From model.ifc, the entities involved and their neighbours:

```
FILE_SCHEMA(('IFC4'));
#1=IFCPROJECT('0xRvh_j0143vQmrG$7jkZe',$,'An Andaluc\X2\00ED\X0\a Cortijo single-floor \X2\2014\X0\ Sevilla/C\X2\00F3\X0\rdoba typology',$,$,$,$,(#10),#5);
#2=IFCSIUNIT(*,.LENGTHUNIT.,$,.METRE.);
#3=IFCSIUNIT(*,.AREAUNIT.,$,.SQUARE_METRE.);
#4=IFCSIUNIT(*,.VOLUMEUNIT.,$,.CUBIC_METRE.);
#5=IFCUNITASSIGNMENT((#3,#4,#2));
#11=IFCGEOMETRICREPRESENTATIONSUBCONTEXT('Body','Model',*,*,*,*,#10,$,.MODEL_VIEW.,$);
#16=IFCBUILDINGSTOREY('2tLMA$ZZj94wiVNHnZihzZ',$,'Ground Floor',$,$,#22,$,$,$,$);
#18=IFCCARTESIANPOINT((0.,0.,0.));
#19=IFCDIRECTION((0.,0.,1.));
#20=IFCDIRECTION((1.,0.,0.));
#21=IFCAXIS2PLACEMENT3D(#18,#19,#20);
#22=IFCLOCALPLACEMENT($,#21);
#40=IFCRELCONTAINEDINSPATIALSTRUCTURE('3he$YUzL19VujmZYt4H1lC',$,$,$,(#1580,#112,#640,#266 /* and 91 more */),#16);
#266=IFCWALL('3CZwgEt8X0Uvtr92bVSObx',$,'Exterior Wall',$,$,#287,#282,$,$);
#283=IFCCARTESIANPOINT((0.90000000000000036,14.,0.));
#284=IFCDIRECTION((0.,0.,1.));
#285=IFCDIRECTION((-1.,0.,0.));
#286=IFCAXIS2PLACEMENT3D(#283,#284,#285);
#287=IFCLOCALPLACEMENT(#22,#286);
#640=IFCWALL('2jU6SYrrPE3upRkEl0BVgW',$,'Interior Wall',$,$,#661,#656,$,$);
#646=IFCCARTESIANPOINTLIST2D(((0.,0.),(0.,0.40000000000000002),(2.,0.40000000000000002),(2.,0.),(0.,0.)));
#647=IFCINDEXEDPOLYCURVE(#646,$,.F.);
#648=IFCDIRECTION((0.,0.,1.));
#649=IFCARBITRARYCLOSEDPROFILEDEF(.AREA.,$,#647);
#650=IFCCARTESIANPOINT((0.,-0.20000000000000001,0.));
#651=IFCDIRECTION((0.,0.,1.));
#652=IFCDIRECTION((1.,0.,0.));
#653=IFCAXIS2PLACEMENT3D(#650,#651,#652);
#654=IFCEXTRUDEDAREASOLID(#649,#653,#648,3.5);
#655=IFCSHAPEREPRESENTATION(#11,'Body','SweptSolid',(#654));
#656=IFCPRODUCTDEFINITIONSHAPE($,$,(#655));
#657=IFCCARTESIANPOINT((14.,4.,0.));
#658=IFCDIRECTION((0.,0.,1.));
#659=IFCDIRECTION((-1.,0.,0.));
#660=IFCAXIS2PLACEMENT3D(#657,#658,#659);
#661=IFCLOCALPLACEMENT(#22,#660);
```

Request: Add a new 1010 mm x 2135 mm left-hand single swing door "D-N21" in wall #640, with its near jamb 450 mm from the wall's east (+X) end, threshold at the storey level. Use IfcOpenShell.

```python
import numpy as np
import ifcopenshell
import ifcopenshell.api.feature
import ifcopenshell.api.geometry
import ifcopenshell.api.root
import ifcopenshell.api.spatial
import ifcopenshell.geom
import ifcopenshell.util.element
import ifcopenshell.util.placement
import ifcopenshell.util.representation
import ifcopenshell.util.shape
import ifcopenshell.util.unit

model = ifcopenshell.open("model.ifc")
unit_scale = ifcopenshell.util.unit.calculate_unit_scale(model)
settings = ifcopenshell.geom.settings()


def volume(element):
    """Net volume in cubic metres, openings subtracted."""
    shape = ifcopenshell.geom.create_shape(settings, element)
    return ifcopenshell.util.shape.get_volume(shape.geometry)


wall = model.by_guid("2jU6SYrrPE3upRkEl0BVgW")
storey = ifcopenshell.util.element.get_container(wall, ifc_class="IfcBuildingStorey")
context = ifcopenshell.util.representation.get_context(model, "Model", "Body", "MODEL_VIEW")
before = volume(wall)

width, height, from_end, sill = 1.01, 2.135, 0.45, 0.0  # metres

# The wall runs along its own X axis, and the end named is its -X end.
wall_shape = ifcopenshell.geom.create_shape(settings, wall)
x, y, z = ifcopenshell.util.shape.get_vertices(wall_shape.geometry).T
start = x.min() + from_end
face, thickness = float(y.min()), float(y.max() - y.min())
wall_matrix = ifcopenshell.util.placement.get_local_placement(wall.ObjectPlacement)
level = ifcopenshell.util.placement.get_local_placement(storey.ObjectPlacement)[2, 3]


def in_wall(x, y):
    """Placement at x, y metres in the wall's axes, at sill height."""
    matrix = wall_matrix.copy()
    matrix[:, 3] = wall_matrix @ np.array([x / unit_scale, y / unit_scale, 0.0, 1.0])
    matrix[2, 3] = level + sill / unit_scale
    return matrix


# Opening: a box that overshoots both wall faces by 50 mm.
opening = ifcopenshell.api.root.create_entity(model, ifc_class="IfcOpeningElement", predefined_type="OPENING")
box = ifcopenshell.api.geometry.add_wall_representation(
    model, context=context, length=width, height=height, thickness=thickness + 0.1
)
ifcopenshell.api.geometry.assign_representation(model, product=opening, representation=box)
ifcopenshell.api.geometry.edit_object_placement(model, product=opening, matrix=in_wall(start, face - 0.05), is_si=False)
ifcopenshell.api.feature.add_feature(model, feature=opening, element=wall)

door = ifcopenshell.api.root.create_entity(model, ifc_class="IfcDoor", name="D-N21", predefined_type="DOOR")
door.OverallWidth, door.OverallHeight = width / unit_scale, height / unit_scale
door.OperationType = "SINGLE_SWING_LEFT"
body = ifcopenshell.api.geometry.add_door_representation(
    model,
    context=context,
    overall_width=door.OverallWidth,
    overall_height=door.OverallHeight,
    operation_type="SINGLE_SWING_LEFT",
    lining_properties={"LiningDepth": thickness / unit_scale, "ThresholdDepth": thickness / unit_scale},
)
ifcopenshell.api.geometry.assign_representation(model, product=door, representation=body)
ifcopenshell.api.spatial.assign_container(model, products=[door], relating_structure=storey)
ifcopenshell.api.feature.add_filling(model, opening=opening, element=door)

# The lining spans the wall, so the door starts at the wall face.
ifcopenshell.api.geometry.edit_object_placement(model, product=door, matrix=in_wall(start, face), is_si=False)

after = volume(wall)

print(f"wall volume {before:.3f} -> {after:.3f} m3")

model.write("model-out.ifc")
```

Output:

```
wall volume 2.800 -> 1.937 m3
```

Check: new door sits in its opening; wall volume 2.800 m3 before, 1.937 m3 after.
